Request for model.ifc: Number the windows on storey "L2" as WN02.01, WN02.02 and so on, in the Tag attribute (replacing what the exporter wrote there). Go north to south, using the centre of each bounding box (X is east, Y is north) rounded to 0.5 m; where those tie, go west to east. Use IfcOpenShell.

First a look at what the model holds.

```python
import ifcopenshell
import ifcopenshell.util.element
import ifcopenshell.util.placement

model = ifcopenshell.open("model.ifc")
print(model.schema)
storey = next(s for s in model.by_type("IfcBuildingStorey") if s.Name == "L2")
windows = [e for e in ifcopenshell.util.element.get_decomposition(storey) if e.is_a("IfcWindow")]
for e in sorted(windows, key=lambda e: e.id()):
    origin = ifcopenshell.util.placement.get_local_placement(e.ObjectPlacement)[:3, 3]
    print(e.id(), e.Tag, e.Name, origin.round(2) + 0.0, sep=" | ")
```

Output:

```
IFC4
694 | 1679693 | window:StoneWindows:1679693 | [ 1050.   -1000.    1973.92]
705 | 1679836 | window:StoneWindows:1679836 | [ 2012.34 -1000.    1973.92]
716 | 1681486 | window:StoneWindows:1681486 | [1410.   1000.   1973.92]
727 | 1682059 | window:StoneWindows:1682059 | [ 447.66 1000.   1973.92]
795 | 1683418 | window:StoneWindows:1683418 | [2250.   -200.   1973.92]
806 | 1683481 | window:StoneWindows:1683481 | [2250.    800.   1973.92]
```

```python
import ifcopenshell
import ifcopenshell.geom
import ifcopenshell.util.element
import ifcopenshell.util.shape

model = ifcopenshell.open("model.ifc")
settings = ifcopenshell.geom.settings()
settings.set("use-world-coords", True)


def centre(element):
    shape = ifcopenshell.geom.create_shape(settings, element)
    return ifcopenshell.util.shape.get_bbox_centroid(shape.geometry)


storey = next(s for s in model.by_type("IfcBuildingStorey") if s.Name == "L2")
windows = [e for e in ifcopenshell.util.element.get_decomposition(storey) if e.is_a("IfcWindow")]

# Insertion points can sit at a corner or the storey origin, so sort by the geometry (in metres).
centres = {e: centre(e) for e in windows}
windows.sort(key=lambda e: (-round(centres[e][1] / 0.5), centres[e][0]))

for i, e in enumerate(windows, start=1):
    number = f"WN02.{i:02d}"
    e.Tag = number
    print(e.id(), number)

model.write("model_edited.ifc")
```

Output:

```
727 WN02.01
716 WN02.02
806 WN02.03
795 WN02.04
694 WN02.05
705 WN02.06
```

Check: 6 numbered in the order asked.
